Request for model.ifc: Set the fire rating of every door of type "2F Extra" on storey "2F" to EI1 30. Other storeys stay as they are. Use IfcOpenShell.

First a look at what the model holds.

```python
import ifcopenshell
import ifcopenshell.util.element

model = ifcopenshell.open("model.ifc")
print(model.schema)
storey = next(s for s in model.by_type("IfcBuildingStorey") if s.Name == "2F")
doors = [e for e in ifcopenshell.util.element.get_decomposition(storey) if e.is_a("IfcDoor")]
seen = {}
for e in doors:
    element_type = ifcopenshell.util.element.get_type(e)
    key = (element_type.Name if element_type != e and element_type else None, ifcopenshell.util.element.get_pset(e, "Pset_DoorCommon", "FireRating"))
    seen[key] = seen.get(key, 0) + 1
for (name, value), count in sorted(seen.items(), key=str):
    print(count, "x", name, "|", value)
```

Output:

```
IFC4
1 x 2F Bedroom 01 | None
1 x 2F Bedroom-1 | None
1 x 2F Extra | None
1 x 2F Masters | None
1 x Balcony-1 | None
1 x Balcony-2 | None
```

```python
import ifcopenshell
import ifcopenshell.api.pset
import ifcopenshell.util.element

model = ifcopenshell.open("model.ifc")

storey = next(s for s in model.by_type("IfcBuildingStorey") if s.Name == "2F")
doors = [e for e in ifcopenshell.util.element.get_decomposition(storey) if e.is_a("IfcDoor")]

count = 0
for e in doors:
    element_type = ifcopenshell.util.element.get_type(e)
    if element_type in (None, e) or element_type.Name != "2F Extra":
        continue
    # add_pset returns the element's existing set when there is one.
    pset = ifcopenshell.api.pset.add_pset(model, product=e, name="Pset_DoorCommon")
    ifcopenshell.api.pset.edit_pset(model, pset=pset, properties={"FireRating": "EI1 30"})
    count += 1

print(count, "doors updated")

model.write("model_edited.ifc")
```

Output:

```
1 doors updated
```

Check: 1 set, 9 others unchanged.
